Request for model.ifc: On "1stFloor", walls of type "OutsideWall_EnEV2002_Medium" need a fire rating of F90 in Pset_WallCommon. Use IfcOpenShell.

First a look at what the model holds.

```python
import ifcopenshell
import ifcopenshell.util.element

model = ifcopenshell.open("model.ifc")
print(model.schema)
storey = next(s for s in model.by_type("IfcBuildingStorey") if s.Name == "1stFloor")
walls = [e for e in ifcopenshell.util.element.get_decomposition(storey) if e.is_a("IfcWall")]
seen = {}
for e in walls:
    element_type = ifcopenshell.util.element.get_type(e)
    key = (element_type.Name if element_type != e and element_type else None, ifcopenshell.util.element.get_pset(e, "Pset_WallCommon", "FireRating"))
    seen[key] = seen.get(key, 0) + 1
for (name, value), count in sorted(seen.items(), key=str):
    print(count, "x", name, "|", value)
```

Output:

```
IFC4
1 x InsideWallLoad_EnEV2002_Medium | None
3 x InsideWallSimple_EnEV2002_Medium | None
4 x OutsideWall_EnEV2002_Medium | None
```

```python
import ifcopenshell
import ifcopenshell.api.pset
import ifcopenshell.util.element

model = ifcopenshell.open("model.ifc")

storey = next(s for s in model.by_type("IfcBuildingStorey") if s.Name == "1stFloor")
walls = [e for e in ifcopenshell.util.element.get_decomposition(storey) if e.is_a("IfcWall")]

count = 0
for e in walls:
    element_type = ifcopenshell.util.element.get_type(e)
    if element_type in (None, e) or element_type.Name != "OutsideWall_EnEV2002_Medium":
        continue
    # add_pset returns the element's existing set when there is one.
    pset = ifcopenshell.api.pset.add_pset(model, product=e, name="Pset_WallCommon")
    ifcopenshell.api.pset.edit_pset(model, pset=pset, properties={"FireRating": "F90"})
    count += 1

print(count, "walls updated")

model.write("model_edited.ifc")
```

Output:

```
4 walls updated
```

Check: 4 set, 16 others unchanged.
